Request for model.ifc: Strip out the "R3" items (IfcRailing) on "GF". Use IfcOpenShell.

First a look at what the model holds.

```python
import ifcopenshell
import ifcopenshell.util.element

model = ifcopenshell.open("model.ifc")
print(model.schema)
storey = next(s for s in model.by_type("IfcBuildingStorey") if s.Name == "GF")
railings = [e for e in ifcopenshell.util.element.get_decomposition(storey) if e.is_a("IfcRailing")]
seen = {}
for e in railings:
    element_type = ifcopenshell.util.element.get_type(e)
    name = element_type.Name if element_type not in (None, e) else None
    seen[name] = seen.get(name, 0) + 1
for name, count in sorted(seen.items(), key=str):
    print(count, "x", name)
```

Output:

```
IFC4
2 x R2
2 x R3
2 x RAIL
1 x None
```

```python
import ifcopenshell
import ifcopenshell.api.root
import ifcopenshell.util.element

model = ifcopenshell.open("model.ifc")

storey = next(s for s in model.by_type("IfcBuildingStorey") if s.Name == "GF")
railings = [e for e in ifcopenshell.util.element.get_decomposition(storey) if e.is_a("IfcRailing")]
targets = [e for e in railings if (t := ifcopenshell.util.element.get_type(e)) not in (None, e) and t.Name == "R3"]

for e in targets:
    ifcopenshell.api.root.remove_product(model, product=e)
print(len(targets), "removed")

model.write("model_rev.ifc")
```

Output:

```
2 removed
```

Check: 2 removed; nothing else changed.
